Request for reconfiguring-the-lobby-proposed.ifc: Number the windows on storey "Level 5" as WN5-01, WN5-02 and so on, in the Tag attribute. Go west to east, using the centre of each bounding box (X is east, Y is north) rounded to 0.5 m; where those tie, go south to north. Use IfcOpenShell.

First a look at what the model holds.

```python
import ifcopenshell
import ifcopenshell.util.element
import ifcopenshell.util.placement

model = ifcopenshell.open("reconfiguring-the-lobby-proposed.ifc")
print(model.schema)
storey = next(s for s in model.by_type("IfcBuildingStorey") if s.Name == "Level 5")
windows = [e for e in ifcopenshell.util.element.get_decomposition(storey) if e.is_a("IfcWindow")]
for e in sorted(windows, key=lambda e: e.id()):
    origin = ifcopenshell.util.placement.get_local_placement(e.ObjectPlacement)[:3, 3]
    print(e.id(), e.Tag, e.Name, origin.round(2) + 0.0, sep=" | ")
```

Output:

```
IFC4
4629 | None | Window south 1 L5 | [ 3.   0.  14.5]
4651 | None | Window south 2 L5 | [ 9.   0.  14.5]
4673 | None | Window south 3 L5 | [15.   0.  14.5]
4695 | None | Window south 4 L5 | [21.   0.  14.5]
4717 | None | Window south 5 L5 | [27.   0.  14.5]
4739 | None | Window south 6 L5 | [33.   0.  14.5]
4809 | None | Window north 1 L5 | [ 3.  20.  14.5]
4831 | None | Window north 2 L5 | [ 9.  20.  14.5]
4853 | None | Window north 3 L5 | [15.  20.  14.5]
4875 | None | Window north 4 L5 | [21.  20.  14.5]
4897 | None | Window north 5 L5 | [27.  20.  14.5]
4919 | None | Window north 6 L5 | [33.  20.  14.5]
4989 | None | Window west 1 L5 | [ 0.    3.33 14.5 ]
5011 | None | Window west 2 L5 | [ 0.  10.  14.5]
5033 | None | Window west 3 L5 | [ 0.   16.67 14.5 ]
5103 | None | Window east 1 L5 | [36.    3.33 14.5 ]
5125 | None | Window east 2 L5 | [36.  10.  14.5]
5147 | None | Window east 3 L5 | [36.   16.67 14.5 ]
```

```python
import ifcopenshell
import ifcopenshell.geom
import ifcopenshell.util.element
import ifcopenshell.util.shape

model = ifcopenshell.open("reconfiguring-the-lobby-proposed.ifc")
settings = ifcopenshell.geom.settings()
settings.set("use-world-coords", True)


def centre(element):
    shape = ifcopenshell.geom.create_shape(settings, element)
    return ifcopenshell.util.shape.get_bbox_centroid(shape.geometry)


storey = next(s for s in model.by_type("IfcBuildingStorey") if s.Name == "Level 5")
windows = [e for e in ifcopenshell.util.element.get_decomposition(storey) if e.is_a("IfcWindow")]

# Insertion points can sit at a corner or the storey origin, so sort by the geometry (in metres).
centres = {e: centre(e) for e in windows}
windows.sort(key=lambda e: (round(centres[e][0] / 0.5), centres[e][1]))

for i, e in enumerate(windows, start=1):
    number = f"WN5-{i:02d}"
    e.Tag = number
    print(e.id(), number)

model.write("reconfiguring-the-lobby-proposed_rev.ifc")
```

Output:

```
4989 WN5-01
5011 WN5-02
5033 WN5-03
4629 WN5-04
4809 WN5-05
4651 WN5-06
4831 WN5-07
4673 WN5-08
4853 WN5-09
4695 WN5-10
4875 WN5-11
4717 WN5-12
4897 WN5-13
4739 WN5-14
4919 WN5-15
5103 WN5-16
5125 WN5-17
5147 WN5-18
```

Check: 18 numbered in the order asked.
